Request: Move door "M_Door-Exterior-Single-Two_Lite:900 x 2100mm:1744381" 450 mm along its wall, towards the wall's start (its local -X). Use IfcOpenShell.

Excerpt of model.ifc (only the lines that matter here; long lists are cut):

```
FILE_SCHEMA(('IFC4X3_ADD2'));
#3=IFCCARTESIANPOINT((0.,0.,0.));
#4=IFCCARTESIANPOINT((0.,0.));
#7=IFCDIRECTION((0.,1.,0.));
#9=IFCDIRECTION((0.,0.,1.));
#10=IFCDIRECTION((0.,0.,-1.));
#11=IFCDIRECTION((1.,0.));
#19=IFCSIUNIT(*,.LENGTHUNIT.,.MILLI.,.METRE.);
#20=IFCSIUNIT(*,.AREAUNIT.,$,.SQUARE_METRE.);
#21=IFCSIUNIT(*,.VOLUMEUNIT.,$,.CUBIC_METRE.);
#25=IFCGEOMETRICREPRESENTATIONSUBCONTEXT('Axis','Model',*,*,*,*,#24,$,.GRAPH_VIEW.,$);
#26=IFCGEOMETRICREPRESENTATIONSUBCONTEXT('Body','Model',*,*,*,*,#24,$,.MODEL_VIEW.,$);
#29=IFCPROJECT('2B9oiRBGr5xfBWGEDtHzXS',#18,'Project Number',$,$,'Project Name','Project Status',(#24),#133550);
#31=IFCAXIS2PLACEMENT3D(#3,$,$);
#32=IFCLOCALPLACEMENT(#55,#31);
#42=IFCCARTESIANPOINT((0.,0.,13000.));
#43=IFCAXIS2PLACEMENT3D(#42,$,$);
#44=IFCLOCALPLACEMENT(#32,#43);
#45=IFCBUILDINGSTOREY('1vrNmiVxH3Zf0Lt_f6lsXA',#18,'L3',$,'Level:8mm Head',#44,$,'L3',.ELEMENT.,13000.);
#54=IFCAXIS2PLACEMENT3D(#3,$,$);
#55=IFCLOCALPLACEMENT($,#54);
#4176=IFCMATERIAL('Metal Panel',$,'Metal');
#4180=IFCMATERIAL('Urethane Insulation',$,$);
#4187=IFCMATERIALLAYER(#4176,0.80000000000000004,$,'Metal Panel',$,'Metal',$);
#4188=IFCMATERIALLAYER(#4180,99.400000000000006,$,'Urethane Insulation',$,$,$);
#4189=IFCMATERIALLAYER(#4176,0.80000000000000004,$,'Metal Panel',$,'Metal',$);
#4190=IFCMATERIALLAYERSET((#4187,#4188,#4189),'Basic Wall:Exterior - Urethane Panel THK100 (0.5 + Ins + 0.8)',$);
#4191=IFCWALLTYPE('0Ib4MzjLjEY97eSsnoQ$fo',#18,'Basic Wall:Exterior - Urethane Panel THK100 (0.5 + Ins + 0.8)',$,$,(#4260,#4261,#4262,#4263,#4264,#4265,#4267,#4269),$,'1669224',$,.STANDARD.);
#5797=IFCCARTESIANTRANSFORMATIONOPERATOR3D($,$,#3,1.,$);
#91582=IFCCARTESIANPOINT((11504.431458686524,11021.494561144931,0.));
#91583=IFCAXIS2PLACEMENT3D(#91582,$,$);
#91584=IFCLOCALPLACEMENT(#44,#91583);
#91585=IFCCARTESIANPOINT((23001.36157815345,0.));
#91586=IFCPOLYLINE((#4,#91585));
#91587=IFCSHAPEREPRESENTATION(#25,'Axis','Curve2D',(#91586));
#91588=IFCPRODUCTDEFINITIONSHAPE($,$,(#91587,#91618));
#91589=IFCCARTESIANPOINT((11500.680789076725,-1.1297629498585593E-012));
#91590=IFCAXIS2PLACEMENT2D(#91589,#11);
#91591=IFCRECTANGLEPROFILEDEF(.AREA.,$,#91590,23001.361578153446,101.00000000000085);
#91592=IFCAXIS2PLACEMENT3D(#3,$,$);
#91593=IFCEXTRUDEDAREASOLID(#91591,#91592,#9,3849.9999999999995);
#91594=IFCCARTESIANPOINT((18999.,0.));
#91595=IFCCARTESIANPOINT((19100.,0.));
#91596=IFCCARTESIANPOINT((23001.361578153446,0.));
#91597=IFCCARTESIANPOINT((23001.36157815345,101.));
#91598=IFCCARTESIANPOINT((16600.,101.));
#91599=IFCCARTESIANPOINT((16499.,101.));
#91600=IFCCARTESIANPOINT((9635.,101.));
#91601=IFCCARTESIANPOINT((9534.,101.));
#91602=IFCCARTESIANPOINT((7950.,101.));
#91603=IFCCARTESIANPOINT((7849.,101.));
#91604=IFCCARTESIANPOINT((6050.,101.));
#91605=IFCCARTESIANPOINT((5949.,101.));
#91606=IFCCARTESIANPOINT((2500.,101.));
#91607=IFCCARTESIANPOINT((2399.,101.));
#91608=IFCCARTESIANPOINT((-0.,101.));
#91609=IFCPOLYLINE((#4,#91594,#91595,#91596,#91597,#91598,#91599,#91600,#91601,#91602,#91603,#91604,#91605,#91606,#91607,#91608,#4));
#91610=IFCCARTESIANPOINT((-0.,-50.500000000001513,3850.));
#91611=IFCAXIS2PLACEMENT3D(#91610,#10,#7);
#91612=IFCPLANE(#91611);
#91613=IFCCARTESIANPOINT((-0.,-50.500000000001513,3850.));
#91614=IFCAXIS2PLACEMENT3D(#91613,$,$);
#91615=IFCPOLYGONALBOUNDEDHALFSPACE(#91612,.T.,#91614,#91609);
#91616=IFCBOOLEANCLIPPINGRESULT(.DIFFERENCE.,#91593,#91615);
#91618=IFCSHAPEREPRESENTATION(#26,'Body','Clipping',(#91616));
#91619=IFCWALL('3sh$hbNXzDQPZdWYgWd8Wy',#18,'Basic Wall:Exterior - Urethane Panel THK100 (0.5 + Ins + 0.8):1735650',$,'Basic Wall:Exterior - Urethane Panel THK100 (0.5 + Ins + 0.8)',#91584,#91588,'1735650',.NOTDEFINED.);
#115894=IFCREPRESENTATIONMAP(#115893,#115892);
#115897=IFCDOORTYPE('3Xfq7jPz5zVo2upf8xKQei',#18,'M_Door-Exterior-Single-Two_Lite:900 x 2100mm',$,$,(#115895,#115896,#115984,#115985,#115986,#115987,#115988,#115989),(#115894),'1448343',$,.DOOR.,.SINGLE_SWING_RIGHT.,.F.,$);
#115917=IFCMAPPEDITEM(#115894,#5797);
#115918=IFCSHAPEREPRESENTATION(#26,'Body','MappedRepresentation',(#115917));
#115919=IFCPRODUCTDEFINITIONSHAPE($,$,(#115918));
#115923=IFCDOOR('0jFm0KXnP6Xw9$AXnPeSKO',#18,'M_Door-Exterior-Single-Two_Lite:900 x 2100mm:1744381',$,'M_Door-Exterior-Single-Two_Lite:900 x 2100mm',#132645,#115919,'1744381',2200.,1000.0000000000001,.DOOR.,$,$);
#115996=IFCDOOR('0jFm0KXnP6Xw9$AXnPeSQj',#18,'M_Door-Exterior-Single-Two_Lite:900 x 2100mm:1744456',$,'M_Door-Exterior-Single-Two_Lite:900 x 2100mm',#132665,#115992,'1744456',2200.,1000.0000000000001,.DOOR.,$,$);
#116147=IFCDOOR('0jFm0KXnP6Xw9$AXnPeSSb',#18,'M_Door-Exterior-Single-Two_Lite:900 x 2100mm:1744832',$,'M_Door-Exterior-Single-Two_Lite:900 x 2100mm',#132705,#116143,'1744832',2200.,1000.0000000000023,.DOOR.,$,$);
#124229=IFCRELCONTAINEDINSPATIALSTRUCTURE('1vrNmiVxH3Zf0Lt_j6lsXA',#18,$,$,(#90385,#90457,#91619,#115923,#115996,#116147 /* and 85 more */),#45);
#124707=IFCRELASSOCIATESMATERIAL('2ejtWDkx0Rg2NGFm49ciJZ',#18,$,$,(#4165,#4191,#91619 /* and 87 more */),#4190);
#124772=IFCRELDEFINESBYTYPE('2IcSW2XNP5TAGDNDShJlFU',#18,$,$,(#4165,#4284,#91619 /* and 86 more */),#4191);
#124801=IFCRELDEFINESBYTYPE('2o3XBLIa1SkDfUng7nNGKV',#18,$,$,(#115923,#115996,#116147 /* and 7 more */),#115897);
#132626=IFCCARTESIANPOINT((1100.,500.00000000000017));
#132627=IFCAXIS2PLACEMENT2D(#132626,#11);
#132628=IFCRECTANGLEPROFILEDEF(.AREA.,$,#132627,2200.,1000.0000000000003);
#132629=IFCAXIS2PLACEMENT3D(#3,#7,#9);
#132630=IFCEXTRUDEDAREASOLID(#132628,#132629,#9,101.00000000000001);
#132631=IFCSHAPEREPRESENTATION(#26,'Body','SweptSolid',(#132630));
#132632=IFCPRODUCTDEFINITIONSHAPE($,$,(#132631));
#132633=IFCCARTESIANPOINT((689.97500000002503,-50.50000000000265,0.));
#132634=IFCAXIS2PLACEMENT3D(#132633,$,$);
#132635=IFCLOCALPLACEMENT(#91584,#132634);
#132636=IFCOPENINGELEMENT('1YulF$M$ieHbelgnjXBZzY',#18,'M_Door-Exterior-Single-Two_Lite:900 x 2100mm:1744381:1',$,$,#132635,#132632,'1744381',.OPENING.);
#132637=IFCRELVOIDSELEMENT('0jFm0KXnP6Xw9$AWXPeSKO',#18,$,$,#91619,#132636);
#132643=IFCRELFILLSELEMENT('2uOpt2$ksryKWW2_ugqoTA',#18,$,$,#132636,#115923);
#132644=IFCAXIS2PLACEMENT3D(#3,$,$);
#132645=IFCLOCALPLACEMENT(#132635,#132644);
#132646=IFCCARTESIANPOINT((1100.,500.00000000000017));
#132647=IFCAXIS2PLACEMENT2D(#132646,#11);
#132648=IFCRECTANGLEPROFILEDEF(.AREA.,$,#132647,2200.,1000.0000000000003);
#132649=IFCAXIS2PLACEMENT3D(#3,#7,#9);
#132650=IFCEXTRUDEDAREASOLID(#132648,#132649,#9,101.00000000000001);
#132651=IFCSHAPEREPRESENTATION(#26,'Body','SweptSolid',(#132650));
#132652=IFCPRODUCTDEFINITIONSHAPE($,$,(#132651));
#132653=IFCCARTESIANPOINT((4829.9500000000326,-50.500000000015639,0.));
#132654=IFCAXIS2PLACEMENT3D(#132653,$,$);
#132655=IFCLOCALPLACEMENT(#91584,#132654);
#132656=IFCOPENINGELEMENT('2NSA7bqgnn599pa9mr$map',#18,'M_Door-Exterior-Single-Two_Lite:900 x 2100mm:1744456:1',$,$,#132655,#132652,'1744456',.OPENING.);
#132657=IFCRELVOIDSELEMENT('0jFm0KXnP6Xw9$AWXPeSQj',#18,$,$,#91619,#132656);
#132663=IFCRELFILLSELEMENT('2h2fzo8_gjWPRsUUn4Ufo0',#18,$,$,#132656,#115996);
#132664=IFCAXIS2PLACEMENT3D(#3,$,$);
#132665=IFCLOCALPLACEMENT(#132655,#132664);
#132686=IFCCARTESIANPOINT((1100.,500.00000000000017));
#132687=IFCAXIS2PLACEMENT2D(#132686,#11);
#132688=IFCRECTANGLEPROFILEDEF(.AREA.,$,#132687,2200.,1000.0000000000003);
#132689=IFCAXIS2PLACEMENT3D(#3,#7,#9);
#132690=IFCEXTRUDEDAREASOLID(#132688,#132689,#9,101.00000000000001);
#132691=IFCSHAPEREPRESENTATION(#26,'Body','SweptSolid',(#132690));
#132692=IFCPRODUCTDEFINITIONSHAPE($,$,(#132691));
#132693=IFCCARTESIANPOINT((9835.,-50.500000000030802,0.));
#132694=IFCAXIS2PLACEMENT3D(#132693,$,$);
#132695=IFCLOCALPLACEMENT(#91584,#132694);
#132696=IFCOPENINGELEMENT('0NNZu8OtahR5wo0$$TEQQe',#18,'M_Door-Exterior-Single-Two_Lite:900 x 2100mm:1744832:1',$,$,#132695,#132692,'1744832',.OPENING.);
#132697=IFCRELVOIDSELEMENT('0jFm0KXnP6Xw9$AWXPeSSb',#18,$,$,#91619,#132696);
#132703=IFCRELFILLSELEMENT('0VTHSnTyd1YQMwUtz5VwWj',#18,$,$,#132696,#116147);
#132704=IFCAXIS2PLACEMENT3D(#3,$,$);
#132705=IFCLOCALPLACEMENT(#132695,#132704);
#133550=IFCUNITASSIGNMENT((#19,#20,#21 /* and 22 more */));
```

```python
import ifcopenshell
import ifcopenshell.api.geometry
import ifcopenshell.util.placement
import ifcopenshell.util.unit

model = ifcopenshell.open("model.ifc")
unit_scale = ifcopenshell.util.unit.calculate_unit_scale(model)

door = model.by_guid("0jFm0KXnP6Xw9$AXnPeSKO")
opening = door.FillsVoids[0].RelatingOpeningElement
wall = opening.VoidsElements[0].RelatingBuildingElement

wall_matrix = ifcopenshell.util.placement.get_local_placement(wall.ObjectPlacement)
shift = wall_matrix[:3, 0] * -0.45 / unit_scale
before = ifcopenshell.util.placement.get_local_placement(door.ObjectPlacement)[:3, 3].copy()

# The door is placed relative to its opening, so it follows when the opening moves.
matrix = ifcopenshell.util.placement.get_local_placement(opening.ObjectPlacement)
matrix[:3, 3] += shift
ifcopenshell.api.geometry.edit_object_placement(
    model, product=opening, matrix=matrix, is_si=False, should_transform_children=True
)

after = ifcopenshell.util.placement.get_local_placement(door.ObjectPlacement)[:3, 3]
print("door moved by", (after - before).round(3) + 0.0)

model.write("model_v2.ifc")
```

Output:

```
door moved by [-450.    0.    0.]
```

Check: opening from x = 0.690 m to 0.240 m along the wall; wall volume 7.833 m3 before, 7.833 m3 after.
